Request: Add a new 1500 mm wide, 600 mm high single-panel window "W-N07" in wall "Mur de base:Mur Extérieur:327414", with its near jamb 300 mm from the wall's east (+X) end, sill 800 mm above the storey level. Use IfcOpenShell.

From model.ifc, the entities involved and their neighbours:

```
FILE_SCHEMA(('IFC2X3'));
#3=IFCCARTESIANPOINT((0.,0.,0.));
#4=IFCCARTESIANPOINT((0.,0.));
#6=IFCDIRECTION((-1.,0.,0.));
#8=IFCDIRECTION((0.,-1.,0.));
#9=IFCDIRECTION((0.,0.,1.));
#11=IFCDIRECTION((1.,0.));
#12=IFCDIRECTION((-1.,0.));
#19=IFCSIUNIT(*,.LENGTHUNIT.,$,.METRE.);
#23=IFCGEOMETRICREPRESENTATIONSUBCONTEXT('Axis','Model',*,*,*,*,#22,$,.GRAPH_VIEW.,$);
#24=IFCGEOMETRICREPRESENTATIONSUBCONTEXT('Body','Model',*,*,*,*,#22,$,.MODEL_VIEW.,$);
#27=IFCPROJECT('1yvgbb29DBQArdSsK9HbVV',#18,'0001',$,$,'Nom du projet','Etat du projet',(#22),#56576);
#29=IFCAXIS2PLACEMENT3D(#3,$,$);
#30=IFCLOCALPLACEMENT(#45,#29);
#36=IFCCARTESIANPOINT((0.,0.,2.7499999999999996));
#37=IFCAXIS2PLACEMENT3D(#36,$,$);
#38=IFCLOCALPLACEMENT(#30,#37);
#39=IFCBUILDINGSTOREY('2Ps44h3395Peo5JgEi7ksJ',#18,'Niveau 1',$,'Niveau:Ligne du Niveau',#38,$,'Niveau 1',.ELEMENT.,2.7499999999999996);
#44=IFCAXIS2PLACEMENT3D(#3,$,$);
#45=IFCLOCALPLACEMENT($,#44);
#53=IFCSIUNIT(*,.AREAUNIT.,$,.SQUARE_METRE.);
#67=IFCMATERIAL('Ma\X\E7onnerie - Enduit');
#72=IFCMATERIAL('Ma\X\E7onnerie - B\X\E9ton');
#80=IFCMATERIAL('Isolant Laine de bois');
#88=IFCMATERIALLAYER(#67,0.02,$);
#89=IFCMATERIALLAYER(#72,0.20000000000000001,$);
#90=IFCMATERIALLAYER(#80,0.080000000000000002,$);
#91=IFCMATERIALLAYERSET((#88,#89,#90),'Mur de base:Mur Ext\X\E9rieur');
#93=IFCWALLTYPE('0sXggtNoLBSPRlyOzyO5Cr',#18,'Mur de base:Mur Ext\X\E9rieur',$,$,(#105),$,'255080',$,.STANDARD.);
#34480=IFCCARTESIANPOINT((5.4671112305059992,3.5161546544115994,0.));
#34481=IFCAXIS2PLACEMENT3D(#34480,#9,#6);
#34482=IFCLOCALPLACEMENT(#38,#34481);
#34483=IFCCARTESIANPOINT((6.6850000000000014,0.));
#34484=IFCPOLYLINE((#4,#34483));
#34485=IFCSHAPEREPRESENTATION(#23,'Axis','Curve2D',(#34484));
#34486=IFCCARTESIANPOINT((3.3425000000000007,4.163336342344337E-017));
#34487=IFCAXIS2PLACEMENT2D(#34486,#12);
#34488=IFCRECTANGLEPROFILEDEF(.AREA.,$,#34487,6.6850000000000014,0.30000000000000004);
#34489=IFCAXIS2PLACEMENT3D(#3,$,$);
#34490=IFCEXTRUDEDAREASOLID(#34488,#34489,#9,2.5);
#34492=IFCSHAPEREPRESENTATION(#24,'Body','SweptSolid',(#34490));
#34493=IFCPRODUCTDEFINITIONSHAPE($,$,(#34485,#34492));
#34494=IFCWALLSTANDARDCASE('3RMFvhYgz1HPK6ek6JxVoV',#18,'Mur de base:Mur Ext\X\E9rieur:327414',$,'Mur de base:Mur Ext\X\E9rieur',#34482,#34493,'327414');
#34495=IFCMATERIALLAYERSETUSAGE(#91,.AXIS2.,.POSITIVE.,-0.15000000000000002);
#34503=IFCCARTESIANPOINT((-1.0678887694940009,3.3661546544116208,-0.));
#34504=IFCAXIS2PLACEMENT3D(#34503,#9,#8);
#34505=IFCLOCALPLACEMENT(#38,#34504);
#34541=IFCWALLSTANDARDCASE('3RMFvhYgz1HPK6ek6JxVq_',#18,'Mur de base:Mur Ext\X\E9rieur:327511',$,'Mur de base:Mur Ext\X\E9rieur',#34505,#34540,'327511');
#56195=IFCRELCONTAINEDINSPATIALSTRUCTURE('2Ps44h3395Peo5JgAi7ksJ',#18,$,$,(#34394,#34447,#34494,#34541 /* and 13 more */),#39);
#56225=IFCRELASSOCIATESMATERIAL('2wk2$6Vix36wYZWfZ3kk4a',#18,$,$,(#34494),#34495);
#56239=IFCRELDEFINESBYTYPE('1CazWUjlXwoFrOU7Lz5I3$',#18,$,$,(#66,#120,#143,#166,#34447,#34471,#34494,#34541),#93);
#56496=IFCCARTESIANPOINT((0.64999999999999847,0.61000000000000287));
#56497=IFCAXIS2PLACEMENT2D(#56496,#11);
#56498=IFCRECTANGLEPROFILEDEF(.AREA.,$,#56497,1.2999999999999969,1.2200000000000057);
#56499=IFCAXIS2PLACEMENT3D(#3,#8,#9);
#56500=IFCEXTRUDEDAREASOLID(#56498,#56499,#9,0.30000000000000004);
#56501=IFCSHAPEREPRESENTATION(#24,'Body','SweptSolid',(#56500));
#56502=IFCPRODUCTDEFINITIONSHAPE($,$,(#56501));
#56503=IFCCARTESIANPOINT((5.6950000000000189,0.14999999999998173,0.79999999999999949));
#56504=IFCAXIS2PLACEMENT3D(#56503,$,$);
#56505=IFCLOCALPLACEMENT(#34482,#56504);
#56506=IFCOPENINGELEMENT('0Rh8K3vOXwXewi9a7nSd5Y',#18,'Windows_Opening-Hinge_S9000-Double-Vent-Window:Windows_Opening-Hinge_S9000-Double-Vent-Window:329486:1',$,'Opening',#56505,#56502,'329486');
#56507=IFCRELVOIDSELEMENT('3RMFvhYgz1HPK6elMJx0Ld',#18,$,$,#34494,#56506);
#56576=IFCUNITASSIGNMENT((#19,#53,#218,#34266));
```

```python
import numpy as np
import ifcopenshell
import ifcopenshell.api.feature
import ifcopenshell.api.geometry
import ifcopenshell.api.root
import ifcopenshell.api.spatial
import ifcopenshell.api.type
import ifcopenshell.geom
import ifcopenshell.util.element
import ifcopenshell.util.placement
import ifcopenshell.util.representation
import ifcopenshell.util.shape
import ifcopenshell.util.unit

model = ifcopenshell.open("model.ifc")
unit_scale = ifcopenshell.util.unit.calculate_unit_scale(model)
settings = ifcopenshell.geom.settings()


def volume(element):
    """Net volume in cubic metres, openings subtracted."""
    shape = ifcopenshell.geom.create_shape(settings, element)
    return ifcopenshell.util.shape.get_volume(shape.geometry)


wall = model.by_guid("3RMFvhYgz1HPK6ek6JxVoV")
storey = ifcopenshell.util.element.get_container(wall, ifc_class="IfcBuildingStorey")
context = ifcopenshell.util.representation.get_context(model, "Model", "Body", "MODEL_VIEW")
before = volume(wall)

width, height, from_end, sill = 1.5, 0.6, 0.3, 0.8  # metres

# The wall runs along its own X axis, and the end named is its -X end.
wall_shape = ifcopenshell.geom.create_shape(settings, wall)
x, y, z = ifcopenshell.util.shape.get_vertices(wall_shape.geometry).T
start = x.min() + from_end
face, thickness = float(y.min()), float(y.max() - y.min())
wall_matrix = ifcopenshell.util.placement.get_local_placement(wall.ObjectPlacement)
level = ifcopenshell.util.placement.get_local_placement(storey.ObjectPlacement)[2, 3]


def in_wall(x, y):
    """Placement at x, y metres in the wall's axes, at sill height."""
    matrix = wall_matrix.copy()
    matrix[:, 3] = wall_matrix @ np.array([x / unit_scale, y / unit_scale, 0.0, 1.0])
    matrix[2, 3] = level + sill / unit_scale
    return matrix


# Opening: a box that overshoots both wall faces by 50 mm.
opening = ifcopenshell.api.root.create_entity(model, ifc_class="IfcOpeningElement")
box = ifcopenshell.api.geometry.add_wall_representation(
    model, context=context, length=width, height=height, thickness=thickness + 0.1
)
ifcopenshell.api.geometry.assign_representation(model, product=opening, representation=box)
ifcopenshell.api.geometry.edit_object_placement(model, product=opening, matrix=in_wall(start, face - 0.05), is_si=False)
ifcopenshell.api.feature.add_feature(model, feature=opening, element=wall)

window = ifcopenshell.api.root.create_entity(model, ifc_class="IfcWindow", name="W-N07")
window.OverallWidth, window.OverallHeight = width / unit_scale, height / unit_scale
body = ifcopenshell.api.geometry.add_window_representation(
    model,
    context=context,
    overall_width=window.OverallWidth,
    overall_height=window.OverallHeight,
    partition_type="SINGLE_PANEL",
)
ifcopenshell.api.geometry.assign_representation(model, product=window, representation=body)
ifcopenshell.api.spatial.assign_container(model, products=[window], relating_structure=storey)
fills = ifcopenshell.api.feature.add_filling(model, opening=opening, element=window)
fills.OwnerHistory = window.OwnerHistory  # required in IFC2X3

# IFC2X3 keeps the operation on the window style.
style = ifcopenshell.api.root.create_entity(model, ifc_class="IfcWindowStyle", name="W-N07")
style.OperationType, style.ConstructionType = "SINGLE_PANEL", "NOTDEFINED"
style.ParameterTakesPrecedence = style.Sizeable = False
ifcopenshell.api.type.assign_type(model, related_objects=[window], relating_type=style)

# Centre the window in the wall's thickness.
ifcopenshell.api.geometry.edit_object_placement(model, product=window, matrix=in_wall(start, face), is_si=False)
window_shape = ifcopenshell.geom.create_shape(settings, window)
depth = ifcopenshell.util.shape.get_vertices(window_shape.geometry)[:, 1]
offset = face + thickness / 2 - (depth.min() + depth.max()) / 2
ifcopenshell.api.geometry.edit_object_placement(model, product=window, matrix=in_wall(start, offset), is_si=False)

after = volume(wall)

print(f"wall volume {before:.3f} -> {after:.3f} m3")

model.write("model_updated.ifc")
```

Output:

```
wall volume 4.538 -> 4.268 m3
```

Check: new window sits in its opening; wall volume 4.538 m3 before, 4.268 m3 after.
